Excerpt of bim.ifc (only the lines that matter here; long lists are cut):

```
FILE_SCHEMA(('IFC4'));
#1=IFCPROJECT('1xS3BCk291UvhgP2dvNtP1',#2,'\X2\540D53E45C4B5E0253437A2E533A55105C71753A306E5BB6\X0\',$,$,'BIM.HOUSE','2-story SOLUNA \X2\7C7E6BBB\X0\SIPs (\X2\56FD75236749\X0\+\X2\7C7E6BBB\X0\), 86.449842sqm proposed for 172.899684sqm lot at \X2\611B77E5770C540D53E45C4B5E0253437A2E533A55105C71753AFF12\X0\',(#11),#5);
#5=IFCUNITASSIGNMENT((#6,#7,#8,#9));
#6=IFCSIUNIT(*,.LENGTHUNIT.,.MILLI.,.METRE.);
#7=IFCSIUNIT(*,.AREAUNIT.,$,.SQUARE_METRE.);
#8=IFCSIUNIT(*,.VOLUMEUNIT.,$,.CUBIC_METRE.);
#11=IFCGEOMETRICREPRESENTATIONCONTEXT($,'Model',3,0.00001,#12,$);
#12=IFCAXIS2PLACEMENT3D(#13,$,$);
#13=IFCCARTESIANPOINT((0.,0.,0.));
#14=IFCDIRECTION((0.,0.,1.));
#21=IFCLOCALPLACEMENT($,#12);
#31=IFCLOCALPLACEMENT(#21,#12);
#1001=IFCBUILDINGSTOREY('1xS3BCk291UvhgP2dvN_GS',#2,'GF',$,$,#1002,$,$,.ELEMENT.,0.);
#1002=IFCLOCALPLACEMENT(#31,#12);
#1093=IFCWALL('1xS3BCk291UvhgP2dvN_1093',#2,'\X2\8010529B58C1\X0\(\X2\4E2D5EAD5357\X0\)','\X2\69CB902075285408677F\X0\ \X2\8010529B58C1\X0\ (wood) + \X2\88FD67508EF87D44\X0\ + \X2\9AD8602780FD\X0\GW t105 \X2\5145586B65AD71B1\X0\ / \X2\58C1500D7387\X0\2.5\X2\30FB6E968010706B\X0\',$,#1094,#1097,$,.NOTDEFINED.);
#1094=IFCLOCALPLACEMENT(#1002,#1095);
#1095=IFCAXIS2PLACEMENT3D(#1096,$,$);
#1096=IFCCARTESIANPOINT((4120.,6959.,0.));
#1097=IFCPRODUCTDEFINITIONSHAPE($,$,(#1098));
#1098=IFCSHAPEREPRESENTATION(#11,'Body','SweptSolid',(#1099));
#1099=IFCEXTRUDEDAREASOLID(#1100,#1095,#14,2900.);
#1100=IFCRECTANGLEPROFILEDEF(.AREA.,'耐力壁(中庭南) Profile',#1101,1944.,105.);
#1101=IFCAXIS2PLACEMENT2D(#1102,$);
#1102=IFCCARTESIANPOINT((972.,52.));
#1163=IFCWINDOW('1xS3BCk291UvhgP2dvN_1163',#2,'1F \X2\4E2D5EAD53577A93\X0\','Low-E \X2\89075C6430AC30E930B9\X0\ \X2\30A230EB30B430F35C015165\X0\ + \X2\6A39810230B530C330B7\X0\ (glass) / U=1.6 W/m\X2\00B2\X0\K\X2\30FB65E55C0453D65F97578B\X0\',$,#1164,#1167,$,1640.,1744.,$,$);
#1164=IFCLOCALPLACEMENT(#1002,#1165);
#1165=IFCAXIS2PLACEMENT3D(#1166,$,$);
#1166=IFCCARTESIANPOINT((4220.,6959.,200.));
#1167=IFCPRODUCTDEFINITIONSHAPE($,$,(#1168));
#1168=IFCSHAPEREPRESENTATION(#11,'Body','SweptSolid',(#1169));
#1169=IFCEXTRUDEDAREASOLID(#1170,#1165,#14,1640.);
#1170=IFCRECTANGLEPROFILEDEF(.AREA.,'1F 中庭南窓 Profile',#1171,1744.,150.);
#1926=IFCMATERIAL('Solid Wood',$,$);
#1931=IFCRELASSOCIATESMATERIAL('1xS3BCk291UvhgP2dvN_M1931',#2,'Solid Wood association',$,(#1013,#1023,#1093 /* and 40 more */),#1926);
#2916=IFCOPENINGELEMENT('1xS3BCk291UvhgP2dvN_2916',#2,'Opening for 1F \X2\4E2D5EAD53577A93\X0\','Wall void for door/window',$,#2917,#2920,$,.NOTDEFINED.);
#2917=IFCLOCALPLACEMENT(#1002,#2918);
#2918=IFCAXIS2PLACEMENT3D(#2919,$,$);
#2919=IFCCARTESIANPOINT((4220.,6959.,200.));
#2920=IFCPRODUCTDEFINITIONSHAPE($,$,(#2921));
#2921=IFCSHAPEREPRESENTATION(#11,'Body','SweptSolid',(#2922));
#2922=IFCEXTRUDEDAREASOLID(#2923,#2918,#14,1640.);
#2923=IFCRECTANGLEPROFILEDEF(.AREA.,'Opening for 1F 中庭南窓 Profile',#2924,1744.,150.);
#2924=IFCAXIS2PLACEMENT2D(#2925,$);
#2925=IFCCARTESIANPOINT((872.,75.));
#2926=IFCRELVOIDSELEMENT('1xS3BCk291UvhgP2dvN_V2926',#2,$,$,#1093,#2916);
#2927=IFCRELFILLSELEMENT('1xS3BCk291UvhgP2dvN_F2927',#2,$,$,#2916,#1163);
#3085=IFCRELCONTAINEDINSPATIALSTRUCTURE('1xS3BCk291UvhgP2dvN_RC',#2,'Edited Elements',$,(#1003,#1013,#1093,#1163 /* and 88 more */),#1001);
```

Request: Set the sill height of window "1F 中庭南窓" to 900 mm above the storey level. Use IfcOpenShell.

```python
import numpy as np
import ifcopenshell
import ifcopenshell.api.geometry
import ifcopenshell.geom
import ifcopenshell.util.element
import ifcopenshell.util.placement
import ifcopenshell.util.shape
import ifcopenshell.util.unit

model = ifcopenshell.open("bim.ifc")
unit_scale = ifcopenshell.util.unit.calculate_unit_scale(model)

window = model.by_guid("1xS3BCk291UvhgP2dvN_1163")
opening = window.FillsVoids[0].RelatingOpeningElement
storey = ifcopenshell.util.element.get_container(window, ifc_class="IfcBuildingStorey")
level = ifcopenshell.util.placement.get_local_placement(storey.ObjectPlacement)[2, 3]

# The opening's origin need not be at the sill, so measure its lowest point.
shape = ifcopenshell.geom.create_shape(ifcopenshell.geom.settings(), opening)
bottom = ifcopenshell.util.shape.get_shape_bottom_elevation(shape, shape.geometry) / unit_scale
dz = level + 900.0 - bottom

shift = np.array([0.0, 0.0, dz])
# The window is not placed relative to its opening, so move both.
for product in (opening, window):
    matrix = ifcopenshell.util.placement.get_local_placement(product.ObjectPlacement)
    matrix[:3, 3] += shift
    ifcopenshell.api.geometry.edit_object_placement(model, product=product, matrix=matrix, is_si=False)

print(f"moved by {dz * unit_scale:+.3f} m")

model.write("bim_v2.ifc")
```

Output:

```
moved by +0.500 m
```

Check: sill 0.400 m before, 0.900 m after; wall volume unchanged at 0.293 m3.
